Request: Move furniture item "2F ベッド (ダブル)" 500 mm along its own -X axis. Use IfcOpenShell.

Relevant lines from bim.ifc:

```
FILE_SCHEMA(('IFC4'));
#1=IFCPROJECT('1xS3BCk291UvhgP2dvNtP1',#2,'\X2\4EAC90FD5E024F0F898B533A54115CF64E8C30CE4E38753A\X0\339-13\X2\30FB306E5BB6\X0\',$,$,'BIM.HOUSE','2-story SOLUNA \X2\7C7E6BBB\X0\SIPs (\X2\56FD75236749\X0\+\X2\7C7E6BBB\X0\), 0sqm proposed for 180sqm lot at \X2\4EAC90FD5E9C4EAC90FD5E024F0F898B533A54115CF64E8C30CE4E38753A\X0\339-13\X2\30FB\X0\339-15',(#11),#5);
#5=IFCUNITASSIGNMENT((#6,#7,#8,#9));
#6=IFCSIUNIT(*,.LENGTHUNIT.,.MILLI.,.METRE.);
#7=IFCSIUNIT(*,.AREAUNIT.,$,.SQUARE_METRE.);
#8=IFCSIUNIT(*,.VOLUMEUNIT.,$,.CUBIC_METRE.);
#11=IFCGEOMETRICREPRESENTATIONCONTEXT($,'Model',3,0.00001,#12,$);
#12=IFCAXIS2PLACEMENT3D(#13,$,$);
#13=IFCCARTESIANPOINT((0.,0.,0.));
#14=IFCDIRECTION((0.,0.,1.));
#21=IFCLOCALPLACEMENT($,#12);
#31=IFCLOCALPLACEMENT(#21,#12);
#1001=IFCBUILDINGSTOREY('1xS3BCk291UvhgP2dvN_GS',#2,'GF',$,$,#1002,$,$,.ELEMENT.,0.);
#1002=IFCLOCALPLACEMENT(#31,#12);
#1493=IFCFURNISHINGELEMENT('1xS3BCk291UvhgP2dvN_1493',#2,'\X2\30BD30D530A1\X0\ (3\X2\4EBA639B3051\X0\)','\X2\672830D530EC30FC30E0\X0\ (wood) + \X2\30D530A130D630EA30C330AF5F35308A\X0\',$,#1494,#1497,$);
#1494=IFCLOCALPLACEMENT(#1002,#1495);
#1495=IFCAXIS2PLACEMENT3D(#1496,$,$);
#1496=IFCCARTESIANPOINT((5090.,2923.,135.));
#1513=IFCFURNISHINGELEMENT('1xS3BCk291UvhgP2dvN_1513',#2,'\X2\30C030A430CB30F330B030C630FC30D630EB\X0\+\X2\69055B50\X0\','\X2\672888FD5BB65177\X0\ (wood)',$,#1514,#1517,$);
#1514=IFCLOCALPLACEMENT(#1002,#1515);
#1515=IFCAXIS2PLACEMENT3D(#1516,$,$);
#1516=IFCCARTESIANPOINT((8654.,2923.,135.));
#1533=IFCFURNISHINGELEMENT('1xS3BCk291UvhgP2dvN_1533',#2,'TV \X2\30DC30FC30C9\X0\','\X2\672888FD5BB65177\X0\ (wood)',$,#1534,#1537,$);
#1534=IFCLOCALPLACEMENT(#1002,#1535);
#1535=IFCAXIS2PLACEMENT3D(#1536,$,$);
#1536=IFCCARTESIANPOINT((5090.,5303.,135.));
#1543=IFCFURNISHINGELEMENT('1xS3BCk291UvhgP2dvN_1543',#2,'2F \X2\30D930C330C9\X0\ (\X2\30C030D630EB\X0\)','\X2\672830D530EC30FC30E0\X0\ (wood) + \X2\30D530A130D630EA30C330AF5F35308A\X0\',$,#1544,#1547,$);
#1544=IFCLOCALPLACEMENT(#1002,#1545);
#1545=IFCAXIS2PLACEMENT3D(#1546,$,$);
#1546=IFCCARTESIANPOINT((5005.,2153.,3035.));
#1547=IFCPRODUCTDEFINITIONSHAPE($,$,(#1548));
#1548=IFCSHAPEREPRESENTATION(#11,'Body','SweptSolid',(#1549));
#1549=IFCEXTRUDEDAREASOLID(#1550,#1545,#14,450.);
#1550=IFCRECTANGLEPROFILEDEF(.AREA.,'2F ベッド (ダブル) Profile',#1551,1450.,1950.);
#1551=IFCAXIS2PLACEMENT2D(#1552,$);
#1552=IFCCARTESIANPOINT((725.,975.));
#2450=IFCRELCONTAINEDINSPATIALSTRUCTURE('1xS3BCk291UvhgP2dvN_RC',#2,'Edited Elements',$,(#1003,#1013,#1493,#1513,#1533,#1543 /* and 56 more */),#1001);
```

```python
import ifcopenshell
import ifcopenshell.api.geometry
import ifcopenshell.util.placement
import ifcopenshell.util.unit

model = ifcopenshell.open("bim.ifc")
unit_scale = ifcopenshell.util.unit.calculate_unit_scale(model)

item = model.by_guid("1xS3BCk291UvhgP2dvN_1543")
matrix = ifcopenshell.util.placement.get_local_placement(item.ObjectPlacement)
matrix[:3, 3] -= matrix[:3, 0] * 0.5 / unit_scale
ifcopenshell.api.geometry.edit_object_placement(model, product=item, matrix=matrix, is_si=False)

print(ifcopenshell.util.placement.get_local_placement(item.ObjectPlacement).round(3) + 0.0)

model.write("bim_updated.ifc")
```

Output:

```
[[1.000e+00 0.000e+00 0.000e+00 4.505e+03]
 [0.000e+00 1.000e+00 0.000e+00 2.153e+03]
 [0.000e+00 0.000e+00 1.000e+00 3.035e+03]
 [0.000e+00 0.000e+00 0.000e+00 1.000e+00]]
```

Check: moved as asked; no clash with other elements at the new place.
